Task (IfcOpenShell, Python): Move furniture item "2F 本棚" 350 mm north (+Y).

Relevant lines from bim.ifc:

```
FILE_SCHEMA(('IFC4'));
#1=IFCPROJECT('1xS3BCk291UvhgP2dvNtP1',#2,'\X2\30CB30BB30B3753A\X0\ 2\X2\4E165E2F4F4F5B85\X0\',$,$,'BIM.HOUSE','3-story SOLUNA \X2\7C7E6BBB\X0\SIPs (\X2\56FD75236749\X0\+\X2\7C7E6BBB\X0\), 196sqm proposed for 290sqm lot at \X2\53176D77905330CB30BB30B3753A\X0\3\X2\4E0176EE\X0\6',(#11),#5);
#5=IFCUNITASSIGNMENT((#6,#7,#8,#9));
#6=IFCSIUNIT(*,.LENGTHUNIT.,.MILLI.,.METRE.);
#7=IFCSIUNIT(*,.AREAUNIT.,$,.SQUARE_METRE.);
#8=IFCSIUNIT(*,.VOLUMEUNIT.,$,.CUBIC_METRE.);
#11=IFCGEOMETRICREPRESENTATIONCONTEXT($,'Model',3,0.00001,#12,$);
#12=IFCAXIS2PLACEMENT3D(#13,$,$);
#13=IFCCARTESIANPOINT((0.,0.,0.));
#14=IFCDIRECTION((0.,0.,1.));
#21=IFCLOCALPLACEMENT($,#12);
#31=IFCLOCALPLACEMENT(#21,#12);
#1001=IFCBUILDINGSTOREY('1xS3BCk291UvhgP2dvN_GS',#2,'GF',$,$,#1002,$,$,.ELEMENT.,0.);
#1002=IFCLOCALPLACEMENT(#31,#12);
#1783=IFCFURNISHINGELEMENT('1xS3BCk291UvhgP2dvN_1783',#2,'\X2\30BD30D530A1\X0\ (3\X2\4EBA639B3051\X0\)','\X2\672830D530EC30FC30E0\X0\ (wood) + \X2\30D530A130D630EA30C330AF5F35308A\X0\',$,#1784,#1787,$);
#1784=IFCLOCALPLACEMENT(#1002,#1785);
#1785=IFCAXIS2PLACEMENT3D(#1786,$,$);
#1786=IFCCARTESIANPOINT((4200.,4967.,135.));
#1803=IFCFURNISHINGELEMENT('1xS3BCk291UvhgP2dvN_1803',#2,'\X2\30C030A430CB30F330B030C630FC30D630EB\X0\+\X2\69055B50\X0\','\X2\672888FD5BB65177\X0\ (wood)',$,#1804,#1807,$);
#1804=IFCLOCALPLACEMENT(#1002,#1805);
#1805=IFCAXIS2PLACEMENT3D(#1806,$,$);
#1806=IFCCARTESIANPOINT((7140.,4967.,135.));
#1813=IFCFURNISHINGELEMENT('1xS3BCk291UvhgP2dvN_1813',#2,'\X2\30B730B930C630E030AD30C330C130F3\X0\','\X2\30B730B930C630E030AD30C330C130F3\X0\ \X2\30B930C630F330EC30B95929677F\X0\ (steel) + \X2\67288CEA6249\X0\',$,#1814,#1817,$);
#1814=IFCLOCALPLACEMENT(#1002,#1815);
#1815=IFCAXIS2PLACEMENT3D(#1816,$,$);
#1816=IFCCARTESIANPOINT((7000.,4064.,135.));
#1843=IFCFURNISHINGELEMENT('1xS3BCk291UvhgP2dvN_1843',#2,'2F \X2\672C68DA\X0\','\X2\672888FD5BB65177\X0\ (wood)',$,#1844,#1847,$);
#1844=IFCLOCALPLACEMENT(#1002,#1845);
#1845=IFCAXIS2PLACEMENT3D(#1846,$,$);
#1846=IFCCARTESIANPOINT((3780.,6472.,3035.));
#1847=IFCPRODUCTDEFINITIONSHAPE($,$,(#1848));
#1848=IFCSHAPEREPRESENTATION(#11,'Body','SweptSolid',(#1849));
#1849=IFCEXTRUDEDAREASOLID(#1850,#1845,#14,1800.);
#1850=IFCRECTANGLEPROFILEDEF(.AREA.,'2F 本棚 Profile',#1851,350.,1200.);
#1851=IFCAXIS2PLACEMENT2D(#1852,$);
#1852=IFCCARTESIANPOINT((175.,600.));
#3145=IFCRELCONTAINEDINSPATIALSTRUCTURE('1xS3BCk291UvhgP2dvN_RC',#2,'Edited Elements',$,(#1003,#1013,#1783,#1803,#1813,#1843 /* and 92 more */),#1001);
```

```python
import ifcopenshell
import ifcopenshell.api.geometry
import ifcopenshell.util.placement
import ifcopenshell.util.unit

model = ifcopenshell.open("bim.ifc")
unit_scale = ifcopenshell.util.unit.calculate_unit_scale(model)

item = model.by_id(1843)
matrix = ifcopenshell.util.placement.get_local_placement(item.ObjectPlacement)
matrix[1, 3] += 0.35 / unit_scale
ifcopenshell.api.geometry.edit_object_placement(model, product=item, matrix=matrix, is_si=False)

print(ifcopenshell.util.placement.get_local_placement(item.ObjectPlacement).round(3) + 0.0)

model.write("bim-out.ifc")
```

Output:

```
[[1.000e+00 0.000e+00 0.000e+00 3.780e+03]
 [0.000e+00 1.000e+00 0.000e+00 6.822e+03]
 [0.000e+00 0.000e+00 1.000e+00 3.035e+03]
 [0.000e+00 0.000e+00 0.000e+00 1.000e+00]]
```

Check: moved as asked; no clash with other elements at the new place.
